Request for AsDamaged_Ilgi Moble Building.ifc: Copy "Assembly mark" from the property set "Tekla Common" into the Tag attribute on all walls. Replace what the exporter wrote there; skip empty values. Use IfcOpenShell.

First a look at what the model holds.

```python
import ifcopenshell
import ifcopenshell.util.element

model = ifcopenshell.open("AsDamaged_Ilgi Moble Building.ifc")
print(model.schema)
walls = model.by_type("IfcWall")
print(len(walls), "walls")
for e in walls[:8]:
    source = ifcopenshell.util.element.get_pset(e, "Tekla Common", "Assembly mark")
    target = e.Tag
    print(e.id(), repr(source), repr(target), sep=" | ")
```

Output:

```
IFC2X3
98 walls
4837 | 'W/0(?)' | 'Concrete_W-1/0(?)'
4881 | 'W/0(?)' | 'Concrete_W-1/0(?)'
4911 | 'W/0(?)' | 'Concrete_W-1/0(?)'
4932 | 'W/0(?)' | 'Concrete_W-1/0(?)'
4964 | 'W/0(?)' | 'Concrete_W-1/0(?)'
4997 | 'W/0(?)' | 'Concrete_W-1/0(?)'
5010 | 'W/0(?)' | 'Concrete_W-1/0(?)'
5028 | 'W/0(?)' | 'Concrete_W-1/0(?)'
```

```python
import ifcopenshell
import ifcopenshell.util.element

model = ifcopenshell.open("AsDamaged_Ilgi Moble Building.ifc")

count = 0
for e in model.by_type("IfcWall"):
    value = ifcopenshell.util.element.get_pset(e, "Tekla Common", "Assembly mark")
    current = e.Tag
    if not value or not value.strip() or current == value:
        continue
    e.Tag = value
    count += 1

print(count, "walls updated")

model.write("AsDamaged_Ilgi Moble Building_v2.ifc")
```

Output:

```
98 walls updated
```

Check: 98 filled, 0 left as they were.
